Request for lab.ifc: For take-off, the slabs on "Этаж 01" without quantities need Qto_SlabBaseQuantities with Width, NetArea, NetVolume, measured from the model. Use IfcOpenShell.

First a look at what the model holds.

```python
import ifcopenshell
import ifcopenshell.util.element
import ifcopenshell.util.unit

model = ifcopenshell.open("lab.ifc")
print(model.schema)
for unit_type in ("LENGTHUNIT", "AREAUNIT", "VOLUMEUNIT"):
    print(unit_type, ifcopenshell.util.unit.calculate_unit_scale(model, unit_type))
storey = next(s for s in model.by_type("IfcBuildingStorey") if s.Name == "Этаж 01")
slabs = [e for e in ifcopenshell.util.element.get_decomposition(storey) if e.is_a("IfcSlab")]
for e in sorted(slabs, key=lambda e: e.id()):
    print(e.id(), e.is_a(), e.Name, list(ifcopenshell.util.element.get_psets(e, qtos_only=True)), sep=" | ")
```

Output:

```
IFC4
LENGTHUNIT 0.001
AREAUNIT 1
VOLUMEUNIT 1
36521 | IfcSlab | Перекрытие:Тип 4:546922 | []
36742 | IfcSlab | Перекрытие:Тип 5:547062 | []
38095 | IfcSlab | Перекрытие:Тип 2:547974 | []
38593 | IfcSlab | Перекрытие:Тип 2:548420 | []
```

```python
import ifcopenshell
import ifcopenshell.api.pset
import ifcopenshell.geom
import ifcopenshell.util.element
import ifcopenshell.util.shape
import ifcopenshell.util.unit

model = ifcopenshell.open("lab.ifc")
unit_scale = ifcopenshell.util.unit.calculate_unit_scale(model)
area_scale = ifcopenshell.util.unit.calculate_unit_scale(model, "AREAUNIT")
volume_scale = ifcopenshell.util.unit.calculate_unit_scale(model, "VOLUMEUNIT")
settings = ifcopenshell.geom.settings()

storey = next(s for s in model.by_type("IfcBuildingStorey") if s.Name == "Этаж 01")
slabs = [e for e in ifcopenshell.util.element.get_decomposition(storey) if e.is_a("IfcSlab")]

for e in sorted(slabs, key=lambda e: e.id()):
    if ifcopenshell.util.element.get_psets(e, qtos_only=True, should_inherit=False):
        continue
    # Geometry comes back in metres, in the element's own axes.
    shape = ifcopenshell.geom.create_shape(settings, e)
    values = {
        "Width": ifcopenshell.util.shape.get_z(shape.geometry) / unit_scale,
        "NetArea": ifcopenshell.util.shape.get_footprint_area(shape.geometry) / area_scale,
        "NetVolume": ifcopenshell.util.shape.get_volume(shape.geometry) / volume_scale,
    }
    qto = ifcopenshell.api.pset.add_qto(model, product=e, name="Qto_SlabBaseQuantities")
    ifcopenshell.api.pset.edit_qto(model, qto=qto, properties=values)
    print(e.id(), {k: round(v, 3) for k, v in values.items()})

model.write("lab_edited.ifc")
```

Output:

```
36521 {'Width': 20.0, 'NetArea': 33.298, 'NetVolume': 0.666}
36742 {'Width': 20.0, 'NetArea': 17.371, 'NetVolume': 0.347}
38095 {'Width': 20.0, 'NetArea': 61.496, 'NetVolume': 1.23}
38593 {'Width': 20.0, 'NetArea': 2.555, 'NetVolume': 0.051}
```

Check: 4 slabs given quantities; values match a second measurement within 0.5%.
